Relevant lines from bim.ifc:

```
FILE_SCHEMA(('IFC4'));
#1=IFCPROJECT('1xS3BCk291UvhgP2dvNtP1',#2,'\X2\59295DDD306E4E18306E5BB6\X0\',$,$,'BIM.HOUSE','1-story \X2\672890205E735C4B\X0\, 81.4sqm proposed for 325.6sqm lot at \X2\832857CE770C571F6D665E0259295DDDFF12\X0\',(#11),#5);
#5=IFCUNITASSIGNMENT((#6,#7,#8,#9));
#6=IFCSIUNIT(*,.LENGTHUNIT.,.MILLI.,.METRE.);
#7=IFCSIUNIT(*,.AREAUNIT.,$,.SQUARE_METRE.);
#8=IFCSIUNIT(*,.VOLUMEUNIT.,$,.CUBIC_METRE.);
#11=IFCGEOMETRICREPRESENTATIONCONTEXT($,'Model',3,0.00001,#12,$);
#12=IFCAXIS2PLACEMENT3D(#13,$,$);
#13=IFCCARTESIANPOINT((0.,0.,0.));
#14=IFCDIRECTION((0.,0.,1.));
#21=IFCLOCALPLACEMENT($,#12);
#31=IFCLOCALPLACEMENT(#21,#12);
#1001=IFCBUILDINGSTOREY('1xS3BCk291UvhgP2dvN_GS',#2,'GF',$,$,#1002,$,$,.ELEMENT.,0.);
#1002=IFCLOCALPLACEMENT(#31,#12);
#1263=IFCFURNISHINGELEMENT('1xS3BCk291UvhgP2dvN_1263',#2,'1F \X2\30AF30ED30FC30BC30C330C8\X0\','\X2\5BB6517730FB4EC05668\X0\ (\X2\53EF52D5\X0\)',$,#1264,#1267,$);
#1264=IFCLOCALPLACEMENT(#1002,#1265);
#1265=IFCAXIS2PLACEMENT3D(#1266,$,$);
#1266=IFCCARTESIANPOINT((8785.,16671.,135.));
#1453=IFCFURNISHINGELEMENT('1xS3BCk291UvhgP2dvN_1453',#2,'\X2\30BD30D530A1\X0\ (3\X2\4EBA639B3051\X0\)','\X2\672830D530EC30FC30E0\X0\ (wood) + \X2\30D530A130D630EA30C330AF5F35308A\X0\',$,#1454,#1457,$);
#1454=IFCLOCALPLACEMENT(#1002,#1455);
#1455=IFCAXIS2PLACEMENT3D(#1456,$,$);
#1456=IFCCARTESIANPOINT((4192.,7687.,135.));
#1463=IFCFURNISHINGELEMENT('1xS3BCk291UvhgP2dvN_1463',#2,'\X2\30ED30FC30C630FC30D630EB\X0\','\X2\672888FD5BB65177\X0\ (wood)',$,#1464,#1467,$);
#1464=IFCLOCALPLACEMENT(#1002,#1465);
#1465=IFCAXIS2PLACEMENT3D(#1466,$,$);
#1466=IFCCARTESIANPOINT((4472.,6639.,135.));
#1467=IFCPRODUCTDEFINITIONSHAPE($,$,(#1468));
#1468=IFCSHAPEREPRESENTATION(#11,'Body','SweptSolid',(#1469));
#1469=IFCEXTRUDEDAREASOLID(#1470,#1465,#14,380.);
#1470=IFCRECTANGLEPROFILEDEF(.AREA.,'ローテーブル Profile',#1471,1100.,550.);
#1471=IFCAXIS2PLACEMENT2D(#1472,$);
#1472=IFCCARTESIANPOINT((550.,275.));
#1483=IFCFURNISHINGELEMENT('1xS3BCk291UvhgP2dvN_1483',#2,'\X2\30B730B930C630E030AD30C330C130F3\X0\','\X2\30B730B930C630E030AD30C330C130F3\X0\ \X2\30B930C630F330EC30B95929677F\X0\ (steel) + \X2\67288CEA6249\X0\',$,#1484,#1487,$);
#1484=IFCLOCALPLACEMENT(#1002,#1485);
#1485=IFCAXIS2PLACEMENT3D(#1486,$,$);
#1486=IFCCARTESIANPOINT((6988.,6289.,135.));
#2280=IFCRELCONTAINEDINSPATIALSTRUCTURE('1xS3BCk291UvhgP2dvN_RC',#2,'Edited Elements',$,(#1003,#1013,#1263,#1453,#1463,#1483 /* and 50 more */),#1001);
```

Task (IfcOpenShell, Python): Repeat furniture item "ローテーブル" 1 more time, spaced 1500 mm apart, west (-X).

```python
import numpy as np
import ifcopenshell
import ifcopenshell.api.geometry
import ifcopenshell.api.root
import ifcopenshell.util.element
import ifcopenshell.util.placement

model = ifcopenshell.open("bim.ifc")


def reuse_history(source, copy):
    """copy_class also copies each property set's owner history, people and application; keep the originals."""
    for rel in copy.IsDefinedBy:
        if rel.is_a("IfcRelDefinesByProperties") and (history := rel.RelatingPropertyDefinition.OwnerHistory):
            rel.RelatingPropertyDefinition.OwnerHistory = source.OwnerHistory
            ifcopenshell.util.element.remove_deep2(model, history)


source = model.by_guid("1xS3BCk291UvhgP2dvN_1463")
base = ifcopenshell.util.placement.get_local_placement(source.ObjectPlacement)
step = np.array([-1.0, 0.0, 0.0]) * 1500.0

for i in range(1, 2):
    copy = ifcopenshell.api.root.copy_class(model, product=source)
    copy.Representation = ifcopenshell.util.element.copy_deep(
        model, source.Representation, exclude=["IfcGeometricRepresentationContext", "IfcRepresentationMap"]
    )
    reuse_history(source, copy)
    matrix = base.copy()
    matrix[:3, 3] += i * step
    print("added at", matrix[:3, 3].round(3) + 0.0)
    ifcopenshell.api.geometry.edit_object_placement(model, product=copy, matrix=matrix, is_si=False)

model.write("bim_rev.ifc")
```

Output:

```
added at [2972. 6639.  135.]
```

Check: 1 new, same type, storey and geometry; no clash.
